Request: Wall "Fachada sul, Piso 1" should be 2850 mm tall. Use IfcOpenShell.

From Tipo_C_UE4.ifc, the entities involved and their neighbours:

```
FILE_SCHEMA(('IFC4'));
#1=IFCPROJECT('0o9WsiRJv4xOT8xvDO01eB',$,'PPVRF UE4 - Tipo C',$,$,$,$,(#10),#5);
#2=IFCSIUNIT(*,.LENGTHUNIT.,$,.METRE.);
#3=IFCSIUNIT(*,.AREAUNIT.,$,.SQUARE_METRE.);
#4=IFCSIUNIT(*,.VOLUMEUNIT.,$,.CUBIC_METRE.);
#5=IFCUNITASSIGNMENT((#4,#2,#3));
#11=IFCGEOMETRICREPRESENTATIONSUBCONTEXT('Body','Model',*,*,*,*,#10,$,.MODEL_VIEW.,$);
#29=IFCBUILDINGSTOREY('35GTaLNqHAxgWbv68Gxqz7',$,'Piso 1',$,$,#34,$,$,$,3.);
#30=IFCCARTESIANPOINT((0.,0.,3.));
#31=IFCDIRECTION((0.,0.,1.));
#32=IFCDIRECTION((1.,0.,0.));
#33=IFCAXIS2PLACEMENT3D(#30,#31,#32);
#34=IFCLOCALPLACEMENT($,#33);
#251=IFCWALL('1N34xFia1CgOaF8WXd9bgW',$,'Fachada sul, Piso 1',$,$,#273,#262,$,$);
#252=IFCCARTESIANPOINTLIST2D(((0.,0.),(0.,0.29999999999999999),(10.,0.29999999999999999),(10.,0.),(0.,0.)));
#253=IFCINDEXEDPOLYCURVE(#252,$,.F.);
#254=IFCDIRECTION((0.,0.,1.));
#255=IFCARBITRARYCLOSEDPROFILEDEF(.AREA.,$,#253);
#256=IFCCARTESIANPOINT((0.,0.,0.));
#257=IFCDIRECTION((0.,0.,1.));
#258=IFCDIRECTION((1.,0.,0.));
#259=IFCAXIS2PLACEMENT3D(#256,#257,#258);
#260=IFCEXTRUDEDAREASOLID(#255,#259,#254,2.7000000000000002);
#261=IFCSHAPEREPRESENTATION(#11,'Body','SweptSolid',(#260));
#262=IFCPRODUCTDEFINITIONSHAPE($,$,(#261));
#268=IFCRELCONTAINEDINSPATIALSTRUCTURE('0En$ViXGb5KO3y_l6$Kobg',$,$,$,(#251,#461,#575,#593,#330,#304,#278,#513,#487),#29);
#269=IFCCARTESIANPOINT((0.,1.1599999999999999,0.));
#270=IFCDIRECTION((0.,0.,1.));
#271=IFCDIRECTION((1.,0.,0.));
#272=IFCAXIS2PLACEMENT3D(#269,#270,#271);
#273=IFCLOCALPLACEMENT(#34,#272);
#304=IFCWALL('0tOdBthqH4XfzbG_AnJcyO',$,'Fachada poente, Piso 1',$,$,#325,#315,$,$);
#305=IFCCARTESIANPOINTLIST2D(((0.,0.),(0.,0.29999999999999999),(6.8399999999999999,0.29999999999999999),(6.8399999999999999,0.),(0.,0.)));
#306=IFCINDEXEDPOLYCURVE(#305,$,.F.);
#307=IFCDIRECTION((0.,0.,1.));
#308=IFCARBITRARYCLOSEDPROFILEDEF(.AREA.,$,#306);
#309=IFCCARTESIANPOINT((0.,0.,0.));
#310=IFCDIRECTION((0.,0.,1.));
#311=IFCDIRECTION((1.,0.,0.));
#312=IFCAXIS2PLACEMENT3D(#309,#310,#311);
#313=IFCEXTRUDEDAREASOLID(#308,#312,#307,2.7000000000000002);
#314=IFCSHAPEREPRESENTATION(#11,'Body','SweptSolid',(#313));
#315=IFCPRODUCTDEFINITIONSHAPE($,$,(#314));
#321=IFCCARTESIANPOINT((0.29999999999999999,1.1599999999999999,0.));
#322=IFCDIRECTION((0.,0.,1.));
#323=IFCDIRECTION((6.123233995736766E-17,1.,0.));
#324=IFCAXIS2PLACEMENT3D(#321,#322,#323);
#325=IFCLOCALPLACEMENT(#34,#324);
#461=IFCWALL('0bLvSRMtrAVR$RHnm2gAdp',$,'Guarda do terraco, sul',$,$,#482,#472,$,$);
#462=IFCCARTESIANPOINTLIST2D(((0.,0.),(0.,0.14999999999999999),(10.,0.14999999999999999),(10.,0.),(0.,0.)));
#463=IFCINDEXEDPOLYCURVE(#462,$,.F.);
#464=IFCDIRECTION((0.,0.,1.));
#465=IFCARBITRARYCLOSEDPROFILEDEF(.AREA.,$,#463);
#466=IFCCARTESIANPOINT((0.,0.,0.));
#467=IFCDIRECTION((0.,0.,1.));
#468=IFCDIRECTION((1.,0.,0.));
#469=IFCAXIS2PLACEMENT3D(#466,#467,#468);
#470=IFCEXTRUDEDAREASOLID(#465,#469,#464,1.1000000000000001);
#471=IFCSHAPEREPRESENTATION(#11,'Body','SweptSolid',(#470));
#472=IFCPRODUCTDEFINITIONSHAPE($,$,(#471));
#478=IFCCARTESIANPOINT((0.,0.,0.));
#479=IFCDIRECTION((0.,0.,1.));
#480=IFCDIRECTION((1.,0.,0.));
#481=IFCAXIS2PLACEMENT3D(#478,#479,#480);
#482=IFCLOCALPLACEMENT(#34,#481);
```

```python
import ifcopenshell
import ifcopenshell.geom
import ifcopenshell.util.representation
import ifcopenshell.util.shape
import ifcopenshell.util.unit

model = ifcopenshell.open("Tipo_C_UE4.ifc")
unit_scale = ifcopenshell.util.unit.calculate_unit_scale(model)
settings = ifcopenshell.geom.settings()


def volume(element):
    """Net volume in cubic metres, openings subtracted."""
    shape = ifcopenshell.geom.create_shape(settings, element)
    return ifcopenshell.util.shape.get_volume(shape.geometry)


wall = model.by_id(251)
before = volume(wall)

body = ifcopenshell.util.representation.get_representation(wall, "Model", "Body")
solid = body.Items[0]
old_height = solid.Depth
solid.Depth = 2.85 / unit_scale
after = volume(wall)

print(f"height {old_height:g} -> {solid.Depth:g}, volume {before:.3f} -> {after:.3f} m3")

model.write("Tipo_C_UE4_v2.ifc")
```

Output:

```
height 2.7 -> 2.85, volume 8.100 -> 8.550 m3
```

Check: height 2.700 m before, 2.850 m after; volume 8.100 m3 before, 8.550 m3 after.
